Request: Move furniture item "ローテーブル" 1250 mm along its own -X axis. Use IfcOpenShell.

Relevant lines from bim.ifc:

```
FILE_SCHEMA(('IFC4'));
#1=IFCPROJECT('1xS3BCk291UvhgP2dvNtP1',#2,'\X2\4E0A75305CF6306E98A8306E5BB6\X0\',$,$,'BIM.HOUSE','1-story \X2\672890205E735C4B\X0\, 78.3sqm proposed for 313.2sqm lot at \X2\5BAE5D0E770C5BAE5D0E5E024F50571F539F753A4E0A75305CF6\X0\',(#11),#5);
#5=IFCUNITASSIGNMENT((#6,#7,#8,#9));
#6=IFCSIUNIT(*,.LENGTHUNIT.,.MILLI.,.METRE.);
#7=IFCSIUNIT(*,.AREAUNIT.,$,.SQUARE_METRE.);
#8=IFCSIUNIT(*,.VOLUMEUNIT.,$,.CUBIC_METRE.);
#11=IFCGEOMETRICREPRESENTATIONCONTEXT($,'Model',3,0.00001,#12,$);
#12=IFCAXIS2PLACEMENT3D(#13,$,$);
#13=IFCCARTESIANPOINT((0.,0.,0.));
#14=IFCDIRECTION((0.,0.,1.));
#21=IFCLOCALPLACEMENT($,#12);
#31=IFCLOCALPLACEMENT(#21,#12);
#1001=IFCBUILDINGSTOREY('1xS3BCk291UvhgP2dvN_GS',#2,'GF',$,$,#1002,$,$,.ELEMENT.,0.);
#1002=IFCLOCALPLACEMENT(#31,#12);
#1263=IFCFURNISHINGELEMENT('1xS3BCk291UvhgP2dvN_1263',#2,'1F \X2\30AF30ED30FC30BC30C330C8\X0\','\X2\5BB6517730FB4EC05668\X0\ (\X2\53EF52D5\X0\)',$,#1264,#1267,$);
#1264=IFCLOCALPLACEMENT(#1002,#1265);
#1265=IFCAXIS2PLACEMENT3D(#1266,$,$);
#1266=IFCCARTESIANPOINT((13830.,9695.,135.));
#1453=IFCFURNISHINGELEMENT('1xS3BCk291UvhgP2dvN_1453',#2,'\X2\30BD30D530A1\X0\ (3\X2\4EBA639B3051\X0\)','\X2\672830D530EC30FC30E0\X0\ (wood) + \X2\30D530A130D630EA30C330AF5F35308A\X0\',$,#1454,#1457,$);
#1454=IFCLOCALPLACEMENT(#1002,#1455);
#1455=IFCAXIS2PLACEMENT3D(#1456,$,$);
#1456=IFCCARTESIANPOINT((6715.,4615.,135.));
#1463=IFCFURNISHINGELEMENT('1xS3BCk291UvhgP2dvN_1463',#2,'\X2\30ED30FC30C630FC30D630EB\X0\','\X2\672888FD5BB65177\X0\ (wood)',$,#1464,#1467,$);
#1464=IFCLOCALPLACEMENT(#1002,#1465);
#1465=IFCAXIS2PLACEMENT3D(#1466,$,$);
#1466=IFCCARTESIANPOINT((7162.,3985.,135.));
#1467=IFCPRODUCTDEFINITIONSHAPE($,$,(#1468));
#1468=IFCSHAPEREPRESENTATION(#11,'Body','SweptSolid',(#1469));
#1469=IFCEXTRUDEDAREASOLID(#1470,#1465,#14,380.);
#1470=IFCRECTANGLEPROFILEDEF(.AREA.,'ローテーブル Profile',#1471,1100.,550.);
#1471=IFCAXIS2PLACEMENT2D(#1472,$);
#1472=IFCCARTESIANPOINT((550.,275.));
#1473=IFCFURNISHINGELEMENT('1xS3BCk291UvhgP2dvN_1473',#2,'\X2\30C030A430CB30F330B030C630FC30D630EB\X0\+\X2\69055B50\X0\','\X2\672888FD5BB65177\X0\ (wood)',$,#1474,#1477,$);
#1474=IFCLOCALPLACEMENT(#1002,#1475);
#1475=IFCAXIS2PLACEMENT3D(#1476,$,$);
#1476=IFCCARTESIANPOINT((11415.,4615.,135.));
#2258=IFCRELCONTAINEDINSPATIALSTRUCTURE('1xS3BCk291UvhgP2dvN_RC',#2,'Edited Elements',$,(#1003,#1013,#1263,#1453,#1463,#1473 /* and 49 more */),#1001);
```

```python
import ifcopenshell
import ifcopenshell.api.geometry
import ifcopenshell.util.placement
import ifcopenshell.util.unit

model = ifcopenshell.open("bim.ifc")
unit_scale = ifcopenshell.util.unit.calculate_unit_scale(model)

item = model.by_id(1463)
matrix = ifcopenshell.util.placement.get_local_placement(item.ObjectPlacement)
matrix[:3, 3] -= matrix[:3, 0] * 1.25 / unit_scale
ifcopenshell.api.geometry.edit_object_placement(model, product=item, matrix=matrix, is_si=False)

print(ifcopenshell.util.placement.get_local_placement(item.ObjectPlacement).round(3) + 0.0)

model.write("bim_v2.ifc")
```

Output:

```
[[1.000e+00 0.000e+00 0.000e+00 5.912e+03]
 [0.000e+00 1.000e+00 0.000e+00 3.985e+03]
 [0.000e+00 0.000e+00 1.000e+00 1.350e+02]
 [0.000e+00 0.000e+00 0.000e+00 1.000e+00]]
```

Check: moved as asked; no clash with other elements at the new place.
